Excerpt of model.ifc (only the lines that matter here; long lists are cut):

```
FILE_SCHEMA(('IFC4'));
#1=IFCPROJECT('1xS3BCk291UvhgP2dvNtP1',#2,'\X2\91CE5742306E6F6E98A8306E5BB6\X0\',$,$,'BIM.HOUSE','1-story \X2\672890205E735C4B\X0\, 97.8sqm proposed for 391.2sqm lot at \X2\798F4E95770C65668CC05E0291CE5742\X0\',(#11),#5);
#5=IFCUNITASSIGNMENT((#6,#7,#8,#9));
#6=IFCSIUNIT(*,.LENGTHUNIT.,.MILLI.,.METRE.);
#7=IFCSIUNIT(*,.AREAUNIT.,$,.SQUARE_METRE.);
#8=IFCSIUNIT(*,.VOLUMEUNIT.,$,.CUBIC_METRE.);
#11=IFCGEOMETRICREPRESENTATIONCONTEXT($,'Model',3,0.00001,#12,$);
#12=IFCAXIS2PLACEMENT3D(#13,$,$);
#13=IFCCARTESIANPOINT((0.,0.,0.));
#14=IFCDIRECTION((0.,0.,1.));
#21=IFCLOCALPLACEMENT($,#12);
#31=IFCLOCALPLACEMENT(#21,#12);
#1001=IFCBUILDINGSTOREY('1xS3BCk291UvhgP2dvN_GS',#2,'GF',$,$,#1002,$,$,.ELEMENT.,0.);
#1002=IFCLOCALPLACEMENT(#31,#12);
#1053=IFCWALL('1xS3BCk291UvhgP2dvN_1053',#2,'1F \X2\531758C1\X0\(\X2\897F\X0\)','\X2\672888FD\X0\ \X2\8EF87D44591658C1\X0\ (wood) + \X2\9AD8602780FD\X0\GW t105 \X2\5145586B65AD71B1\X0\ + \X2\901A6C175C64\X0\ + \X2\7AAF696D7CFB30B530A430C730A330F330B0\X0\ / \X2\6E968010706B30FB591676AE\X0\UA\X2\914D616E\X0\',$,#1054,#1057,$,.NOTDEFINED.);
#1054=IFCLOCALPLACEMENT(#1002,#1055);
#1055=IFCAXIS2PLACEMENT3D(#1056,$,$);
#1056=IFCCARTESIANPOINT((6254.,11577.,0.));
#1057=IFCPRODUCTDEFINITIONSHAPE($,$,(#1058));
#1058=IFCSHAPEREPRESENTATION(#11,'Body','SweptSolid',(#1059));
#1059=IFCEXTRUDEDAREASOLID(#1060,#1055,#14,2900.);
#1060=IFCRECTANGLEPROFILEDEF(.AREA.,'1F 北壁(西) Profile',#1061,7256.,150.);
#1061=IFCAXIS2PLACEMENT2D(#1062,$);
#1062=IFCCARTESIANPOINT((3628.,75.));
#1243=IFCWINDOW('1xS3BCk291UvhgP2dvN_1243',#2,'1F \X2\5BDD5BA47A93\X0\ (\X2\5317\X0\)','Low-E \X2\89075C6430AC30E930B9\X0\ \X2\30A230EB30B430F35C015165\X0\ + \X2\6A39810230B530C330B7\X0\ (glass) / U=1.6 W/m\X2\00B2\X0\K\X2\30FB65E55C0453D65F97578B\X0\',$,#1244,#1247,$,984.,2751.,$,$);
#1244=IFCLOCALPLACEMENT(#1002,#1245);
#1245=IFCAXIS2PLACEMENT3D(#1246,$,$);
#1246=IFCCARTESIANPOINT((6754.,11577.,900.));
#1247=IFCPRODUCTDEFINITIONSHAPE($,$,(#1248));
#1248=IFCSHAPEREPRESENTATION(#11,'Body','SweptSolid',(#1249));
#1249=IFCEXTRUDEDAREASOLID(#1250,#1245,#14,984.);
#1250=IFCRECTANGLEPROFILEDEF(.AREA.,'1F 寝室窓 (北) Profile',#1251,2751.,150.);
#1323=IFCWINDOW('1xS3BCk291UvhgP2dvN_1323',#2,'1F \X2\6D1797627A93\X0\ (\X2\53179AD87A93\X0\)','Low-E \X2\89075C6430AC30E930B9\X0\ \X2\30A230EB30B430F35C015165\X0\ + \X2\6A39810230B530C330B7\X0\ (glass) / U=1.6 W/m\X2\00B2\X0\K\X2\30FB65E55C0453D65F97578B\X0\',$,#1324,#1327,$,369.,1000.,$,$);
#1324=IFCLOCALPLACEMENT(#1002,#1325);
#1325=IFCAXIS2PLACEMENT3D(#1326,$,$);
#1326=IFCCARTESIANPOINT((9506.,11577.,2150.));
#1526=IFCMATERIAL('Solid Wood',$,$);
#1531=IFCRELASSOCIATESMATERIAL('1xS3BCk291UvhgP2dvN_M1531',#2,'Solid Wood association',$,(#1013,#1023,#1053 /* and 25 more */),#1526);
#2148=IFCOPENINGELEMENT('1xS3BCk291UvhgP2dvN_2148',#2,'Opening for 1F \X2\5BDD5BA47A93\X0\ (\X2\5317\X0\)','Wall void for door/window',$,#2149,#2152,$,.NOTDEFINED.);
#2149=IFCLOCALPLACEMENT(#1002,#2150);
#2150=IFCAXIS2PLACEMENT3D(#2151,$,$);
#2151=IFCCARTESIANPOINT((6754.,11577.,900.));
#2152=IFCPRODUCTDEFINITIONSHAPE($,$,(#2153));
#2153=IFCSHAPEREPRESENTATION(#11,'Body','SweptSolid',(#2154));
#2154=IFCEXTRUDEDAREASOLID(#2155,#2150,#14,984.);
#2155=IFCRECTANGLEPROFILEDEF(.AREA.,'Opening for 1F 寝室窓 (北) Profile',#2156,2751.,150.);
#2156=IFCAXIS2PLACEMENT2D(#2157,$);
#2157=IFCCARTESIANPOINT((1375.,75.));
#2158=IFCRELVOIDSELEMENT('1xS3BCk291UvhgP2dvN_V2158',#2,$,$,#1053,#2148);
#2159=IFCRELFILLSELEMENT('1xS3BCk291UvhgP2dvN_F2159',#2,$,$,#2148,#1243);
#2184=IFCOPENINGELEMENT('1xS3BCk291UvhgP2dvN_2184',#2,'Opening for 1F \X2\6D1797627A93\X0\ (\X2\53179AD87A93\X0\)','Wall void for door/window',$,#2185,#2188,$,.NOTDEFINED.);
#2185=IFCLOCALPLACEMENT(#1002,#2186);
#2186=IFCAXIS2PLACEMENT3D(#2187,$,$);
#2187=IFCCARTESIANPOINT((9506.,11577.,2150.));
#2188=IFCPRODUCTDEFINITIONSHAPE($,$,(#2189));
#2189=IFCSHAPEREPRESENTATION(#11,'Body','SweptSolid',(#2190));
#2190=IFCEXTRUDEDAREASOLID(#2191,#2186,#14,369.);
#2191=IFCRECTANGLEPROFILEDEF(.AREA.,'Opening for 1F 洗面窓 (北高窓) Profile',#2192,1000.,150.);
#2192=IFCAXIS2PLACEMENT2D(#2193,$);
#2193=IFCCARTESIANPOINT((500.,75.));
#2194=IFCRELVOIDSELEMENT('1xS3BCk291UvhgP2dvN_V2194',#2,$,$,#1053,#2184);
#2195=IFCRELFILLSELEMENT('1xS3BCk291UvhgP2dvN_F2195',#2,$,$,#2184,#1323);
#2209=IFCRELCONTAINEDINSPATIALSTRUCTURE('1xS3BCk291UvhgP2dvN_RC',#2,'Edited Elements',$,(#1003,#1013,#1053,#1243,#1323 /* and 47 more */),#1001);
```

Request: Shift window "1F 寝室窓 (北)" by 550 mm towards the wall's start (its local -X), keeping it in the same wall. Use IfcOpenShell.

```python
import ifcopenshell
import ifcopenshell.api.geometry
import ifcopenshell.util.placement

model = ifcopenshell.open("model.ifc")

window = model.by_guid("1xS3BCk291UvhgP2dvN_1243")
opening = window.FillsVoids[0].RelatingOpeningElement
wall = opening.VoidsElements[0].RelatingBuildingElement

wall_matrix = ifcopenshell.util.placement.get_local_placement(wall.ObjectPlacement)
shift = wall_matrix[:3, 0] * -550.0
before = ifcopenshell.util.placement.get_local_placement(window.ObjectPlacement)[:3, 3].copy()

# The window is not placed relative to its opening, so move both.
for product in (opening, window):
    matrix = ifcopenshell.util.placement.get_local_placement(product.ObjectPlacement)
    matrix[:3, 3] += shift
    ifcopenshell.api.geometry.edit_object_placement(model, product=product, matrix=matrix, is_si=False)

after = ifcopenshell.util.placement.get_local_placement(window.ObjectPlacement)[:3, 3]
print("window moved by", (after - before).round(3) + 0.0)

model.write("model_updated.ifc")
```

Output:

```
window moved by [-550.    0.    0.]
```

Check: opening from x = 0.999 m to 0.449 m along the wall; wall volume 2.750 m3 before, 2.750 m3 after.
